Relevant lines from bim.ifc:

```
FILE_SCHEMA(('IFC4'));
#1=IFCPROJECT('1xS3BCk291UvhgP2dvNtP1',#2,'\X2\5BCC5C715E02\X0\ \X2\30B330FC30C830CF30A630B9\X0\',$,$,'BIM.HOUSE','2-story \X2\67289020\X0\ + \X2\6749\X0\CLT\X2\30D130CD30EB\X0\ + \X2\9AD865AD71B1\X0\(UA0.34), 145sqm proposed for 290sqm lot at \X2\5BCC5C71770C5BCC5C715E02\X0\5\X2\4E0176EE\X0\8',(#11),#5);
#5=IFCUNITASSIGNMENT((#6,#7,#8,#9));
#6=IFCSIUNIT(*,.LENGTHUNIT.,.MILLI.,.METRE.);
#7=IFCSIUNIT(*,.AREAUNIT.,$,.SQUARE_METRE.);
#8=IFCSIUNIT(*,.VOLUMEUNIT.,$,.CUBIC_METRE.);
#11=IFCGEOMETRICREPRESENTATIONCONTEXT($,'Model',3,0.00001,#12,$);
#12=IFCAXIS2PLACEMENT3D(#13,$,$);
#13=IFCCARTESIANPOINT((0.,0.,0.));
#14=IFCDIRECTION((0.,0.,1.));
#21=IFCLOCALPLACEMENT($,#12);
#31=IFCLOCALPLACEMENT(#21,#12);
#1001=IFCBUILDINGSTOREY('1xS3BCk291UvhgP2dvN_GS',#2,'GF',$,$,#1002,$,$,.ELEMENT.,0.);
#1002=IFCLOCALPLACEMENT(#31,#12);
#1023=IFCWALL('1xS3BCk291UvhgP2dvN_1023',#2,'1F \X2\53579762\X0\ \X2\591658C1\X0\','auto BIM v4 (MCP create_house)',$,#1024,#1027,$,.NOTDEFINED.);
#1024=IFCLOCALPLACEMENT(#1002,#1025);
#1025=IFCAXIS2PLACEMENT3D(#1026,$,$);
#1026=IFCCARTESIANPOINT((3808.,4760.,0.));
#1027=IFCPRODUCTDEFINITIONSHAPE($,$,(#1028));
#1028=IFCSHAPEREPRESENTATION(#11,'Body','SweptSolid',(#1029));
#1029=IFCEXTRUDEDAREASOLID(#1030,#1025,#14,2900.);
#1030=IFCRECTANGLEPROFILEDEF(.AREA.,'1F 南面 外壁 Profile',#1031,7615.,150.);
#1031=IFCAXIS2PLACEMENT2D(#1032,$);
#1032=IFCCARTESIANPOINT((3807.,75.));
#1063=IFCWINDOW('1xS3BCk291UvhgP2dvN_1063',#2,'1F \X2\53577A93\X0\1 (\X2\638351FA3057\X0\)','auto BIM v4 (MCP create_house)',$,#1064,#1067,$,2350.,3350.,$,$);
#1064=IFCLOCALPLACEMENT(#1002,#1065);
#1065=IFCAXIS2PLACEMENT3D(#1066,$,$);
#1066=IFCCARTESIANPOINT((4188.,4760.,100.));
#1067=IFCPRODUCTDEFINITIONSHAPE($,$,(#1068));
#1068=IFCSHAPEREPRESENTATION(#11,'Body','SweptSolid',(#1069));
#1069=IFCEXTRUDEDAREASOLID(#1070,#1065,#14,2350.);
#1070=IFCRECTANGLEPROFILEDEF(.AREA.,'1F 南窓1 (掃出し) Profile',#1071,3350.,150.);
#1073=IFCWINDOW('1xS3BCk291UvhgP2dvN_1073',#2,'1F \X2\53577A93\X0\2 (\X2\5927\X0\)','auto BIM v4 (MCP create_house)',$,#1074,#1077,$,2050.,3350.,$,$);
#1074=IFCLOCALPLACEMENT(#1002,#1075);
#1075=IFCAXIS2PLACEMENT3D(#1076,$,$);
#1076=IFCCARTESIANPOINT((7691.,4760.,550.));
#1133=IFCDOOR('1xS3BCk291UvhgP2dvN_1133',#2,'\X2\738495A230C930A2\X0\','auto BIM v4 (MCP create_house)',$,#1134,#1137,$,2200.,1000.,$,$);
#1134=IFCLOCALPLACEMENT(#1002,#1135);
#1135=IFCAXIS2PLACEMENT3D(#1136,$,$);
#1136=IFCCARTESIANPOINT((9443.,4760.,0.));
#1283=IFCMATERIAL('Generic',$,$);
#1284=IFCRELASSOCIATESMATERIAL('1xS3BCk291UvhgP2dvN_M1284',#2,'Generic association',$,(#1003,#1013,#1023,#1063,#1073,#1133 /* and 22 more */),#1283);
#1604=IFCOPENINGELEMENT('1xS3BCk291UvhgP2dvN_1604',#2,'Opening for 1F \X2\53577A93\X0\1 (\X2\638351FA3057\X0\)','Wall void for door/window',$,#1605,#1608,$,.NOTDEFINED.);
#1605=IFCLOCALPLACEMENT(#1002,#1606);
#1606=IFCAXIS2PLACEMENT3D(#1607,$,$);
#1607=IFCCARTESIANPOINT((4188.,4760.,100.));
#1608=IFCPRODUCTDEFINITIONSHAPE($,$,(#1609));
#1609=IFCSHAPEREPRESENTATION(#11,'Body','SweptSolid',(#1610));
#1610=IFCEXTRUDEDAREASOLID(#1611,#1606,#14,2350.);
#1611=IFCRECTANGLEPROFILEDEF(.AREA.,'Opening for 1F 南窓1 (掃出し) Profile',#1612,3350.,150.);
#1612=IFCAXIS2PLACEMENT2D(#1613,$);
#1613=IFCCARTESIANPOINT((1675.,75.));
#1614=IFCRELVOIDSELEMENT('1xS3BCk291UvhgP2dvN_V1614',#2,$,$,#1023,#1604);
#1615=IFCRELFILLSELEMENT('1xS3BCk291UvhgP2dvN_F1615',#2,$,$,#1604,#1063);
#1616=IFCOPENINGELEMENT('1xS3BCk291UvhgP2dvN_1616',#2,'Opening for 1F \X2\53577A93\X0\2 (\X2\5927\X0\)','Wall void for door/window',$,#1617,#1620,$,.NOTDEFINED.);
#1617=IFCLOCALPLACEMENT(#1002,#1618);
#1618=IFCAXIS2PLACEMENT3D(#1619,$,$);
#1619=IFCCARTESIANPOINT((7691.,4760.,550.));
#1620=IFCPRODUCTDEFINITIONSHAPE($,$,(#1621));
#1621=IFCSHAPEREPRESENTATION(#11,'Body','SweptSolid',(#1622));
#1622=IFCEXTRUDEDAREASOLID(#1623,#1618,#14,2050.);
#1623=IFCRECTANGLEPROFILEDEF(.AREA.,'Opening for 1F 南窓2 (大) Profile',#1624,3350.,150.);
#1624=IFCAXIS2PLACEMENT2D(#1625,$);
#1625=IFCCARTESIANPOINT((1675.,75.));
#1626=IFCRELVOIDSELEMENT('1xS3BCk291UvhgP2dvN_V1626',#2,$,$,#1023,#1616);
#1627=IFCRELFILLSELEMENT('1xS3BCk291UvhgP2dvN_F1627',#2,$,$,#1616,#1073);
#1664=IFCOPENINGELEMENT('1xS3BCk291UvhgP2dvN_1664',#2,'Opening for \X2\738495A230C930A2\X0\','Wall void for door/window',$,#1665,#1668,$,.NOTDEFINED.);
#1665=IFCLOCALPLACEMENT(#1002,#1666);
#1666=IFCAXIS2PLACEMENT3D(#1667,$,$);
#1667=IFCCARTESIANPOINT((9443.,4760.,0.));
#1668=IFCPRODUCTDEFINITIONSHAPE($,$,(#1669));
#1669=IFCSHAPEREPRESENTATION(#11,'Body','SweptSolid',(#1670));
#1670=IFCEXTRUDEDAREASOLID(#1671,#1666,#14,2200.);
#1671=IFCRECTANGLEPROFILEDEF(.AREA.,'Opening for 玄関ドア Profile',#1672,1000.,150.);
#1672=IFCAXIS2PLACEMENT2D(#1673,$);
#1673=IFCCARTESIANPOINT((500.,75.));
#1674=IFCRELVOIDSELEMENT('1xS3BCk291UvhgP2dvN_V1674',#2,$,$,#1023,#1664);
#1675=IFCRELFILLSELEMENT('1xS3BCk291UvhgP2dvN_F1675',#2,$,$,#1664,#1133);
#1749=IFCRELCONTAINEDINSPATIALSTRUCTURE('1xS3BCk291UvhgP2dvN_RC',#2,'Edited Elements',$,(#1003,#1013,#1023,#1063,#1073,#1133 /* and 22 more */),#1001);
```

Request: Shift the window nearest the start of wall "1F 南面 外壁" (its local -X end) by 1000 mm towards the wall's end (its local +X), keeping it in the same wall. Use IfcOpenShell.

```python
import ifcopenshell
import ifcopenshell.api.geometry
import ifcopenshell.util.placement

model = ifcopenshell.open("bim.ifc")

window = model.by_guid("1xS3BCk291UvhgP2dvN_1063")
opening = window.FillsVoids[0].RelatingOpeningElement
wall = opening.VoidsElements[0].RelatingBuildingElement

wall_matrix = ifcopenshell.util.placement.get_local_placement(wall.ObjectPlacement)
shift = wall_matrix[:3, 0] * 1000.0
before = ifcopenshell.util.placement.get_local_placement(window.ObjectPlacement)[:3, 3].copy()

# The window is not placed relative to its opening, so move both.
for product in (opening, window):
    matrix = ifcopenshell.util.placement.get_local_placement(product.ObjectPlacement)
    matrix[:3, 3] += shift
    ifcopenshell.api.geometry.edit_object_placement(model, product=product, matrix=matrix, is_si=False)

after = ifcopenshell.util.placement.get_local_placement(window.ObjectPlacement)[:3, 3]
print("window moved by", (after - before).round(3) + 0.0)

model.write("bim_v2.ifc")
```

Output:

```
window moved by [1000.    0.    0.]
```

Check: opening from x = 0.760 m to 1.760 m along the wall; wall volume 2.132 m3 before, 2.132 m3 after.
